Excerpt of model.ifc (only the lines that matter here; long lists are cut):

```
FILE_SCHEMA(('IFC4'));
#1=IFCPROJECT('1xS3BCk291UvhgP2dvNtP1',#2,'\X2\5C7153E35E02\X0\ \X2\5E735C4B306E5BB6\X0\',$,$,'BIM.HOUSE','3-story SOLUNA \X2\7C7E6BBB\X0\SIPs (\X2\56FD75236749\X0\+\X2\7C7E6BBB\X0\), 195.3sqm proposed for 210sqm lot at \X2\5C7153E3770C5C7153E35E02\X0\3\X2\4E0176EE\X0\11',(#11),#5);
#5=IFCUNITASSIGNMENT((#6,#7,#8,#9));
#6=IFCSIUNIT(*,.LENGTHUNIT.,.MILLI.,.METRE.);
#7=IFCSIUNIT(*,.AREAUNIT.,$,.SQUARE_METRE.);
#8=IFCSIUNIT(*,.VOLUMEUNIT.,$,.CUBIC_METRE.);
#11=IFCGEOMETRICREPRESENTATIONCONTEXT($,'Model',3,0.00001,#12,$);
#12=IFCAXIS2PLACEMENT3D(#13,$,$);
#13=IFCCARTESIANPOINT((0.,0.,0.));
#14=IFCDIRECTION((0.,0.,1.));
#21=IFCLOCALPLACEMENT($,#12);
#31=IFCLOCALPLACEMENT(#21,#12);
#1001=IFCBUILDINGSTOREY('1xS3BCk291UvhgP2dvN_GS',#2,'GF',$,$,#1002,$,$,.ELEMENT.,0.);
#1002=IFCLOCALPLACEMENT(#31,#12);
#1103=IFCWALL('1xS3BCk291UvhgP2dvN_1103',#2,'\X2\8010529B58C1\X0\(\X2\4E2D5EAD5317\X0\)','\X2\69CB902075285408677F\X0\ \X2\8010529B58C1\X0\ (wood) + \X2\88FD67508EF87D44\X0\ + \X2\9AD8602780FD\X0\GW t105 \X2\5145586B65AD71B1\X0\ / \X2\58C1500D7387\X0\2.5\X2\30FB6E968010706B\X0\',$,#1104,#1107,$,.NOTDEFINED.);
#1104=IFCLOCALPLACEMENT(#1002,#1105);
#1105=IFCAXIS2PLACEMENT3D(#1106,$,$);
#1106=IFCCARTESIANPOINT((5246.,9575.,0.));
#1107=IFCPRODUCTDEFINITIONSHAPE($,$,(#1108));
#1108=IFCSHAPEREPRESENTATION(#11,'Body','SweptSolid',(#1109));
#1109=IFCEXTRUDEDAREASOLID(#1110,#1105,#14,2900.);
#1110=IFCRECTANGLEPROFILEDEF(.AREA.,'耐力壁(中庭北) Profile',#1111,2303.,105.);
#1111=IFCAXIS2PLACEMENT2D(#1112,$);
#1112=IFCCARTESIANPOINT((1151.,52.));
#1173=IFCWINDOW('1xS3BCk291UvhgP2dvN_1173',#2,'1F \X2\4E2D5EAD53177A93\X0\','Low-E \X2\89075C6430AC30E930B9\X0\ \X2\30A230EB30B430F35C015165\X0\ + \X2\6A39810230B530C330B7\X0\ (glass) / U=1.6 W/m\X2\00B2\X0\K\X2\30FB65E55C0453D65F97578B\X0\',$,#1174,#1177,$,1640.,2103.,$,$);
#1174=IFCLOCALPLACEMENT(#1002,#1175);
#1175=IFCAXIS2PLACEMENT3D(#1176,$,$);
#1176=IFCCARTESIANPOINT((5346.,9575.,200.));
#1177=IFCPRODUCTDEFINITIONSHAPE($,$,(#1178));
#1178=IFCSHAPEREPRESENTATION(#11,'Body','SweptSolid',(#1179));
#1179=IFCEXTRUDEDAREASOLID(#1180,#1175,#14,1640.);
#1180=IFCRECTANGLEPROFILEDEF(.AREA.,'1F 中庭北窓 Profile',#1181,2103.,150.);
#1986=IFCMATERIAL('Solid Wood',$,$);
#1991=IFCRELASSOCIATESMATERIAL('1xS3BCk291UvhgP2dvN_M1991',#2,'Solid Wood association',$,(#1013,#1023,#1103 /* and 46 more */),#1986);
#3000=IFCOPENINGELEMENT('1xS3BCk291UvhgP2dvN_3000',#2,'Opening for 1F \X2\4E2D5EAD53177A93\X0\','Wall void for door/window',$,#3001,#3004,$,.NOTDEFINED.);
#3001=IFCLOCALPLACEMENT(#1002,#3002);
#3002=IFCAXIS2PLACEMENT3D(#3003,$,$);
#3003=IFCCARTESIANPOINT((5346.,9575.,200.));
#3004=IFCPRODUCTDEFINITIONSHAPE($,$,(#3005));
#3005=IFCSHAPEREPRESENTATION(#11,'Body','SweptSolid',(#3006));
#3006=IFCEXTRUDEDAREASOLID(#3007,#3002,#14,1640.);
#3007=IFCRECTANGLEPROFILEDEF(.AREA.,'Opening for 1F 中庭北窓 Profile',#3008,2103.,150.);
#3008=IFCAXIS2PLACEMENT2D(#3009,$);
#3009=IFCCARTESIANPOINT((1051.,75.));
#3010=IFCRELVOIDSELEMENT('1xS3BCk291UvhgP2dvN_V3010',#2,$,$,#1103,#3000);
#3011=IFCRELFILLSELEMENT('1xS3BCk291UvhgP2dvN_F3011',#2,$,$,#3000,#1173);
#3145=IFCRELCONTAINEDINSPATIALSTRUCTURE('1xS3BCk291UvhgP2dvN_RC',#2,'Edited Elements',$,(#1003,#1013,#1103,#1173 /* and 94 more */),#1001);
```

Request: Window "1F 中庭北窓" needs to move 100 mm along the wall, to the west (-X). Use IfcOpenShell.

```python
import ifcopenshell
import ifcopenshell.api.geometry
import ifcopenshell.util.placement

model = ifcopenshell.open("model.ifc")

window = model.by_guid("1xS3BCk291UvhgP2dvN_1173")
opening = window.FillsVoids[0].RelatingOpeningElement
wall = opening.VoidsElements[0].RelatingBuildingElement

wall_matrix = ifcopenshell.util.placement.get_local_placement(wall.ObjectPlacement)
shift = wall_matrix[:3, 0] * -100.0
before = ifcopenshell.util.placement.get_local_placement(window.ObjectPlacement)[:3, 3].copy()

# The window is not placed relative to its opening, so move both.
for product in (opening, window):
    matrix = ifcopenshell.util.placement.get_local_placement(product.ObjectPlacement)
    matrix[:3, 3] += shift
    ifcopenshell.api.geometry.edit_object_placement(model, product=product, matrix=matrix, is_si=False)

after = ifcopenshell.util.placement.get_local_placement(window.ObjectPlacement)[:3, 3]
print("window moved by", (after - before).round(3) + 0.0)

model.write("model_rev.ifc")
```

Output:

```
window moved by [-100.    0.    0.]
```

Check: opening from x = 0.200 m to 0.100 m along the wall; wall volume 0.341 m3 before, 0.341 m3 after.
